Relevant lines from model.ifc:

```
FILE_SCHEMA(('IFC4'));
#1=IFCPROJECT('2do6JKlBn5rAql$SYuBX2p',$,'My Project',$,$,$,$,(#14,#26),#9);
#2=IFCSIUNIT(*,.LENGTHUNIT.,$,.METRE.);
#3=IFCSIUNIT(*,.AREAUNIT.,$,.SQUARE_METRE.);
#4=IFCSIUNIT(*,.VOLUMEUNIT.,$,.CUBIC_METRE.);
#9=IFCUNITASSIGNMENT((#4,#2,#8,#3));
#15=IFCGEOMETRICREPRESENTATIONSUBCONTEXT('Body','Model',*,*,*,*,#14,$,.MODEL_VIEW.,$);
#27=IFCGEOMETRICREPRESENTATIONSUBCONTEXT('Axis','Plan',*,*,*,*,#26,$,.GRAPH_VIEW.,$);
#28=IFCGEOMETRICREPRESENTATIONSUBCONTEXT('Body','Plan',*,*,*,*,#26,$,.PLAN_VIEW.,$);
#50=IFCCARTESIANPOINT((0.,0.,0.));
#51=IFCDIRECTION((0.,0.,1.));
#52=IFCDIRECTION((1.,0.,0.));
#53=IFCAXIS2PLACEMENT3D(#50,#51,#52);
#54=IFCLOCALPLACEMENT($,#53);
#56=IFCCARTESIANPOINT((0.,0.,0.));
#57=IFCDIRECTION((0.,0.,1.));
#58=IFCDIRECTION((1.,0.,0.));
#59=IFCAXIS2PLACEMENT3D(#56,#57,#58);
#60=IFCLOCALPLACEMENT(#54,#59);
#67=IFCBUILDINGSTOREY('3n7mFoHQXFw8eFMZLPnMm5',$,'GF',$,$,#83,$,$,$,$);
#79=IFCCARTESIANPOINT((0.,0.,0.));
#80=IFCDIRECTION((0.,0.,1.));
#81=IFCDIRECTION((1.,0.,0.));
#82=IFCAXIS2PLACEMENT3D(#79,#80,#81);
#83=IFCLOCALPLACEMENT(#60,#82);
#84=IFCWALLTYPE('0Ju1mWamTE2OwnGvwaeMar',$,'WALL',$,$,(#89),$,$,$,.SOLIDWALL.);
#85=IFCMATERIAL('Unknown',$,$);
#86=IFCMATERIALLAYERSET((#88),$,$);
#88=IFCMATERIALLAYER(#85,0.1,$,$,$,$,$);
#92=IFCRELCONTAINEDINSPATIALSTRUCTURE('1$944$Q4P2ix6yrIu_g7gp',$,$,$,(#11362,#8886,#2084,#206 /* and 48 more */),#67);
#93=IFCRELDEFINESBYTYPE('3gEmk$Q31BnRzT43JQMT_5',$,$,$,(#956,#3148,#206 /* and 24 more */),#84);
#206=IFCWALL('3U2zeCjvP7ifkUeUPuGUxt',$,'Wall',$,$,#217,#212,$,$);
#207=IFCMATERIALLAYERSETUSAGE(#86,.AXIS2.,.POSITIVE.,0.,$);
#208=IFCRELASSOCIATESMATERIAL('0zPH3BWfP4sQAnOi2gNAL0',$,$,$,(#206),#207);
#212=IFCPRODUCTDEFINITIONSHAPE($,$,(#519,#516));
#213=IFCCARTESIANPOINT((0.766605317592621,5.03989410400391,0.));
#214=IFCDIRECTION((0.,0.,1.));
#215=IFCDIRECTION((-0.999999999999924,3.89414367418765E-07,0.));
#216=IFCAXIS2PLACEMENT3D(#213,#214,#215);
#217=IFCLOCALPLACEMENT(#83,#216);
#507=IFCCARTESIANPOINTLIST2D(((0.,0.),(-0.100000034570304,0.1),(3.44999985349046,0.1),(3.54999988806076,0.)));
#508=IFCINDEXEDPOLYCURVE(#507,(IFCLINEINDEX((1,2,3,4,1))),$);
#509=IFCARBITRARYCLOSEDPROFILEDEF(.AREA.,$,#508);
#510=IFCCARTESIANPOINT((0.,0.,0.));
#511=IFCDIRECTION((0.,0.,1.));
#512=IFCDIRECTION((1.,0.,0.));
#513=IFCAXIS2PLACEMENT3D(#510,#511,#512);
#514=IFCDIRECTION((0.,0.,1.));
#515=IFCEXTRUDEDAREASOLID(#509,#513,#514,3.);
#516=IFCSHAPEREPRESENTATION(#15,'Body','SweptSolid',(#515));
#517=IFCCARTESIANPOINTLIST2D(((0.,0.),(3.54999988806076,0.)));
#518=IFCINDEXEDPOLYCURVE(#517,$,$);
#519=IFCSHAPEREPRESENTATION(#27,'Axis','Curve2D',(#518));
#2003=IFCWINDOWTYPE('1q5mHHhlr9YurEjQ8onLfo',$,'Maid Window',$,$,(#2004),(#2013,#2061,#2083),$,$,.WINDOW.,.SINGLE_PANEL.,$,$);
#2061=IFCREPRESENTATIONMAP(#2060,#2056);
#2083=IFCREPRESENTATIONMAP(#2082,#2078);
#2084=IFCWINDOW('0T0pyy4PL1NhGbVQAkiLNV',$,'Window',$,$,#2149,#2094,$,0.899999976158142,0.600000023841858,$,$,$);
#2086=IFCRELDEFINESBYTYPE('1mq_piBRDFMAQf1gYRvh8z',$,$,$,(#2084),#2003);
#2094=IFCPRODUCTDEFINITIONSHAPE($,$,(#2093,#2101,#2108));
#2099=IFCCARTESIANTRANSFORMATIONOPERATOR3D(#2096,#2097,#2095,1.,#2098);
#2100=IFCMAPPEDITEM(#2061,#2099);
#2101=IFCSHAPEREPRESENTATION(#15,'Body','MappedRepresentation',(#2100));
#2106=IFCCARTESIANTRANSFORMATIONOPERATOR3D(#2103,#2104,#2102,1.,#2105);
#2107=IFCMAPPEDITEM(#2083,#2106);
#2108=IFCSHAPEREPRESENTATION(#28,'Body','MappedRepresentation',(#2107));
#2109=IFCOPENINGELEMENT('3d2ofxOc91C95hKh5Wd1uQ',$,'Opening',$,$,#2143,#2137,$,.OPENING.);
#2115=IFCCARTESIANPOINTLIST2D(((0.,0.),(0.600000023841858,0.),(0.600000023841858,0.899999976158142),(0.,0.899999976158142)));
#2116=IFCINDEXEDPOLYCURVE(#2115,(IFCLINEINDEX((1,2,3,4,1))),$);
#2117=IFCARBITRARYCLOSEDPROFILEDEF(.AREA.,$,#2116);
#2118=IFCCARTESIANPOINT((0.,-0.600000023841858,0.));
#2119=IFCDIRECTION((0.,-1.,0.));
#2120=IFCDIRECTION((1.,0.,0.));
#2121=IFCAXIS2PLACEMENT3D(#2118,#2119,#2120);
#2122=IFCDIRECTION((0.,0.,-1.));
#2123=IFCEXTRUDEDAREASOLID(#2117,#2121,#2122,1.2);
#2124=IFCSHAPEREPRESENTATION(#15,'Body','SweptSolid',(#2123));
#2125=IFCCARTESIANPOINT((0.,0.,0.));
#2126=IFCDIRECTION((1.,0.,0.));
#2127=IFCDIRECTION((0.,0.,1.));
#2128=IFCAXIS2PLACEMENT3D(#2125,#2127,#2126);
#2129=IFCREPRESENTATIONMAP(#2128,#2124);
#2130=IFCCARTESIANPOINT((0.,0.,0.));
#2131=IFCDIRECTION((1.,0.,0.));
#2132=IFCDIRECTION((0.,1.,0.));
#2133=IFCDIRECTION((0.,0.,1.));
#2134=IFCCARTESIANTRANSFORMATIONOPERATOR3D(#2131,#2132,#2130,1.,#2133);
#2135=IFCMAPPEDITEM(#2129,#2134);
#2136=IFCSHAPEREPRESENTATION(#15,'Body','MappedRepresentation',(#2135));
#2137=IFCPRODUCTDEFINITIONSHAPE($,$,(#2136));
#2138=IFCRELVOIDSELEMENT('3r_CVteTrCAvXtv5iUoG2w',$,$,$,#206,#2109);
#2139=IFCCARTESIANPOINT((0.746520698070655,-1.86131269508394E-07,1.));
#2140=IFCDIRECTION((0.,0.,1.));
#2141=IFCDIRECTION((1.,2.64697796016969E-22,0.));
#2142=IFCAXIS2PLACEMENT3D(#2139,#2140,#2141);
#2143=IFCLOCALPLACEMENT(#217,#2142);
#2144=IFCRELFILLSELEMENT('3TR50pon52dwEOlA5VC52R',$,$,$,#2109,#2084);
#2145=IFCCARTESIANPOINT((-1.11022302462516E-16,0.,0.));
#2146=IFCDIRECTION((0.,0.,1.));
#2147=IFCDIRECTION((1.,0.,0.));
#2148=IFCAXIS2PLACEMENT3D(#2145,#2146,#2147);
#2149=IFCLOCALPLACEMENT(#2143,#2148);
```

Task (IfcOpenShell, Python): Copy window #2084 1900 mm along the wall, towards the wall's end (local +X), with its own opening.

```python
import ifcopenshell
import ifcopenshell.api.feature
import ifcopenshell.api.geometry
import ifcopenshell.api.root
import ifcopenshell.geom
import ifcopenshell.util.element
import ifcopenshell.util.placement
import ifcopenshell.util.shape
import ifcopenshell.util.unit

model = ifcopenshell.open("model.ifc")
unit_scale = ifcopenshell.util.unit.calculate_unit_scale(model)
settings = ifcopenshell.geom.settings()


def volume(element):
    """Net volume in cubic metres, openings subtracted."""
    shape = ifcopenshell.geom.create_shape(settings, element)
    return ifcopenshell.util.shape.get_volume(shape.geometry)


window = model.by_id(2084)
opening = window.FillsVoids[0].RelatingOpeningElement
wall = opening.VoidsElements[0].RelatingBuildingElement
before = volume(wall)
shift = ifcopenshell.util.placement.get_local_placement(wall.ObjectPlacement)[:3, 0] * 1.9 / unit_scale

# copy_class copies the void relationship, type, container and properties, but no geometry.
new_opening = ifcopenshell.api.root.copy_class(model, product=opening)
new_opening.Representation = ifcopenshell.util.element.copy_deep(
    model, opening.Representation, exclude=["IfcGeometricRepresentationContext", "IfcRepresentationMap"]
)
new_window = ifcopenshell.api.root.copy_class(model, product=window)
new_window.Representation = ifcopenshell.util.element.copy_deep(
    model, window.Representation, exclude=["IfcGeometricRepresentationContext", "IfcRepresentationMap"]
)
ifcopenshell.api.feature.add_filling(model, opening=new_opening, element=new_window)

for old, new in ((opening, new_opening), (window, new_window)):
    matrix = ifcopenshell.util.placement.get_local_placement(old.ObjectPlacement)
    matrix[:3, 3] += shift
    ifcopenshell.api.geometry.edit_object_placement(model, product=new, matrix=matrix, is_si=False)

after = volume(wall)

print(f"wall volume {before:.3f} -> {after:.3f} m3")

model.write("model_v2.ifc")
```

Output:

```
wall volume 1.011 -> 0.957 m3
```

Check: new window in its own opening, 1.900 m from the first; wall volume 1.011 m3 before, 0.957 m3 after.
